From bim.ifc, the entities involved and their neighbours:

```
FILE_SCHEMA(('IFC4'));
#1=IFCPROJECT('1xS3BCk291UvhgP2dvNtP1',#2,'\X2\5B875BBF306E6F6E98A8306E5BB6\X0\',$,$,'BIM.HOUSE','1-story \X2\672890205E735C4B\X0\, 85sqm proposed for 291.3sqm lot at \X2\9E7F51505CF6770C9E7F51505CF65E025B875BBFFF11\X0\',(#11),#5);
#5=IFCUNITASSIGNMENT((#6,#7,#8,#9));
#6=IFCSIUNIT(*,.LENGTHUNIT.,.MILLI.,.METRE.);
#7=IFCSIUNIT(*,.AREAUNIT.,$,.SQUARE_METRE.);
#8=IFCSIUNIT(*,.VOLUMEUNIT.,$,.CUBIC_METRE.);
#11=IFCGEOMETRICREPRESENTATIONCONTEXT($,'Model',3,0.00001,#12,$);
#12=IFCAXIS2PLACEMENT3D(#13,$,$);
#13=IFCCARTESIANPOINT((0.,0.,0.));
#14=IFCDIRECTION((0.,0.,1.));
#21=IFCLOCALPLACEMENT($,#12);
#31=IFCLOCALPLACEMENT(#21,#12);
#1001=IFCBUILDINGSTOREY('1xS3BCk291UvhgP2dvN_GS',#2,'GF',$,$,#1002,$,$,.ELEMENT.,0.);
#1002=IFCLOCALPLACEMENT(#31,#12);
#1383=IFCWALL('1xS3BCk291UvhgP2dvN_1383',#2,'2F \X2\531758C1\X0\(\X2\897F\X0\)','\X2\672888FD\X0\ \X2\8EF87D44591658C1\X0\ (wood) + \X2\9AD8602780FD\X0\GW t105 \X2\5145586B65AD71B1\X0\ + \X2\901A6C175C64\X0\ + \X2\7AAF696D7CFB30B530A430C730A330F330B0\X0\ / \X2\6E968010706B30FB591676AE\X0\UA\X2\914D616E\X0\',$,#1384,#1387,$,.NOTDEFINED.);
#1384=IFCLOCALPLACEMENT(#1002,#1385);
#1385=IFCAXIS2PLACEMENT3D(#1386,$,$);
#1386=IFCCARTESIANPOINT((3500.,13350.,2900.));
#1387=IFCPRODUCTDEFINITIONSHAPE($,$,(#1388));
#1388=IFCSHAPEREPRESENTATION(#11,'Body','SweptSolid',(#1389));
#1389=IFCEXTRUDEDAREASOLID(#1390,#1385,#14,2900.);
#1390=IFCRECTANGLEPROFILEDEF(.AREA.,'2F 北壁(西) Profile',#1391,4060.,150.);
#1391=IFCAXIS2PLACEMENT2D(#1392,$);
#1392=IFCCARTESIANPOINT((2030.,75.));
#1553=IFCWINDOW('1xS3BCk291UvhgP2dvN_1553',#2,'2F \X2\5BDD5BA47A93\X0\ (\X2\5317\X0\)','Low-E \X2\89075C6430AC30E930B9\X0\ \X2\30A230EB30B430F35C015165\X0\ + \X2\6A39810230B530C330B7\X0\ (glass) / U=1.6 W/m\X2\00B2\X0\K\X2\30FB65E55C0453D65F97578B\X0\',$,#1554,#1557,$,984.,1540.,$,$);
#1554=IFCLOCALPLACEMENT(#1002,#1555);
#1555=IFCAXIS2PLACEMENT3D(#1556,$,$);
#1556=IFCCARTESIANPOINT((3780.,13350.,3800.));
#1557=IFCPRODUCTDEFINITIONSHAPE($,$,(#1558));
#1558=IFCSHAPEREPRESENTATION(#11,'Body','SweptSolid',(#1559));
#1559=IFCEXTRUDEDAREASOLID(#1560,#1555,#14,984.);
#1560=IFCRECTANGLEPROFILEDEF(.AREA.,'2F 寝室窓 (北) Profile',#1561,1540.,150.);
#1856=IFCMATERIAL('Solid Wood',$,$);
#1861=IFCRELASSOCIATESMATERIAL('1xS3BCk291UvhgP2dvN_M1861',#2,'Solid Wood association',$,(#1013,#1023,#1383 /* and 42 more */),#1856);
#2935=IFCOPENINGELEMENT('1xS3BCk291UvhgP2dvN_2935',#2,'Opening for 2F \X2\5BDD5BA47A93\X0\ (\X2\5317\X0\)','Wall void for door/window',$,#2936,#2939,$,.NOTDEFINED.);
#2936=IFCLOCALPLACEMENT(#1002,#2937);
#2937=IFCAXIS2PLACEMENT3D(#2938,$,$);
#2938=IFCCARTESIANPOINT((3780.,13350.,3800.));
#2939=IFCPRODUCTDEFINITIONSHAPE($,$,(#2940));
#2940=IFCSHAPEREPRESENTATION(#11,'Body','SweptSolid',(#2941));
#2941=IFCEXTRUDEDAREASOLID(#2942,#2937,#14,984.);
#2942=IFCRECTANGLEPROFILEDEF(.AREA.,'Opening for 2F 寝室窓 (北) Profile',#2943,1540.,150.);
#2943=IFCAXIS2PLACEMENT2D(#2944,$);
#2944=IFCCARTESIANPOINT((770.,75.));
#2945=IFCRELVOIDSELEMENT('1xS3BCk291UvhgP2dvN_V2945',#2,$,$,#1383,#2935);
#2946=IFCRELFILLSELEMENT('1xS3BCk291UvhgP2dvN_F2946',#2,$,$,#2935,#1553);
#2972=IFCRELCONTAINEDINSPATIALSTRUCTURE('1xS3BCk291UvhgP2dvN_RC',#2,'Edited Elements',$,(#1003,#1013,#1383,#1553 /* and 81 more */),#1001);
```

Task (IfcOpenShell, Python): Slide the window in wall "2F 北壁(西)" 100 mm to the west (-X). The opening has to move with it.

```python
import ifcopenshell
import ifcopenshell.api.geometry
import ifcopenshell.util.placement
import ifcopenshell.util.unit

model = ifcopenshell.open("bim.ifc")
unit_scale = ifcopenshell.util.unit.calculate_unit_scale(model)

window = model.by_id(1553)
opening = window.FillsVoids[0].RelatingOpeningElement
wall = opening.VoidsElements[0].RelatingBuildingElement

wall_matrix = ifcopenshell.util.placement.get_local_placement(wall.ObjectPlacement)
shift = wall_matrix[:3, 0] * -0.1 / unit_scale
before = ifcopenshell.util.placement.get_local_placement(window.ObjectPlacement)[:3, 3].copy()

# The window is not placed relative to its opening, so move both.
for product in (opening, window):
    matrix = ifcopenshell.util.placement.get_local_placement(product.ObjectPlacement)
    matrix[:3, 3] += shift
    ifcopenshell.api.geometry.edit_object_placement(model, product=product, matrix=matrix, is_si=False)

after = ifcopenshell.util.placement.get_local_placement(window.ObjectPlacement)[:3, 3]
print("window moved by", (after - before).round(3) + 0.0)

model.write("bim_rev.ifc")
```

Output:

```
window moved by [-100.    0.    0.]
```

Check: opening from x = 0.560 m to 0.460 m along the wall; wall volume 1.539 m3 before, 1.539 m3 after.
